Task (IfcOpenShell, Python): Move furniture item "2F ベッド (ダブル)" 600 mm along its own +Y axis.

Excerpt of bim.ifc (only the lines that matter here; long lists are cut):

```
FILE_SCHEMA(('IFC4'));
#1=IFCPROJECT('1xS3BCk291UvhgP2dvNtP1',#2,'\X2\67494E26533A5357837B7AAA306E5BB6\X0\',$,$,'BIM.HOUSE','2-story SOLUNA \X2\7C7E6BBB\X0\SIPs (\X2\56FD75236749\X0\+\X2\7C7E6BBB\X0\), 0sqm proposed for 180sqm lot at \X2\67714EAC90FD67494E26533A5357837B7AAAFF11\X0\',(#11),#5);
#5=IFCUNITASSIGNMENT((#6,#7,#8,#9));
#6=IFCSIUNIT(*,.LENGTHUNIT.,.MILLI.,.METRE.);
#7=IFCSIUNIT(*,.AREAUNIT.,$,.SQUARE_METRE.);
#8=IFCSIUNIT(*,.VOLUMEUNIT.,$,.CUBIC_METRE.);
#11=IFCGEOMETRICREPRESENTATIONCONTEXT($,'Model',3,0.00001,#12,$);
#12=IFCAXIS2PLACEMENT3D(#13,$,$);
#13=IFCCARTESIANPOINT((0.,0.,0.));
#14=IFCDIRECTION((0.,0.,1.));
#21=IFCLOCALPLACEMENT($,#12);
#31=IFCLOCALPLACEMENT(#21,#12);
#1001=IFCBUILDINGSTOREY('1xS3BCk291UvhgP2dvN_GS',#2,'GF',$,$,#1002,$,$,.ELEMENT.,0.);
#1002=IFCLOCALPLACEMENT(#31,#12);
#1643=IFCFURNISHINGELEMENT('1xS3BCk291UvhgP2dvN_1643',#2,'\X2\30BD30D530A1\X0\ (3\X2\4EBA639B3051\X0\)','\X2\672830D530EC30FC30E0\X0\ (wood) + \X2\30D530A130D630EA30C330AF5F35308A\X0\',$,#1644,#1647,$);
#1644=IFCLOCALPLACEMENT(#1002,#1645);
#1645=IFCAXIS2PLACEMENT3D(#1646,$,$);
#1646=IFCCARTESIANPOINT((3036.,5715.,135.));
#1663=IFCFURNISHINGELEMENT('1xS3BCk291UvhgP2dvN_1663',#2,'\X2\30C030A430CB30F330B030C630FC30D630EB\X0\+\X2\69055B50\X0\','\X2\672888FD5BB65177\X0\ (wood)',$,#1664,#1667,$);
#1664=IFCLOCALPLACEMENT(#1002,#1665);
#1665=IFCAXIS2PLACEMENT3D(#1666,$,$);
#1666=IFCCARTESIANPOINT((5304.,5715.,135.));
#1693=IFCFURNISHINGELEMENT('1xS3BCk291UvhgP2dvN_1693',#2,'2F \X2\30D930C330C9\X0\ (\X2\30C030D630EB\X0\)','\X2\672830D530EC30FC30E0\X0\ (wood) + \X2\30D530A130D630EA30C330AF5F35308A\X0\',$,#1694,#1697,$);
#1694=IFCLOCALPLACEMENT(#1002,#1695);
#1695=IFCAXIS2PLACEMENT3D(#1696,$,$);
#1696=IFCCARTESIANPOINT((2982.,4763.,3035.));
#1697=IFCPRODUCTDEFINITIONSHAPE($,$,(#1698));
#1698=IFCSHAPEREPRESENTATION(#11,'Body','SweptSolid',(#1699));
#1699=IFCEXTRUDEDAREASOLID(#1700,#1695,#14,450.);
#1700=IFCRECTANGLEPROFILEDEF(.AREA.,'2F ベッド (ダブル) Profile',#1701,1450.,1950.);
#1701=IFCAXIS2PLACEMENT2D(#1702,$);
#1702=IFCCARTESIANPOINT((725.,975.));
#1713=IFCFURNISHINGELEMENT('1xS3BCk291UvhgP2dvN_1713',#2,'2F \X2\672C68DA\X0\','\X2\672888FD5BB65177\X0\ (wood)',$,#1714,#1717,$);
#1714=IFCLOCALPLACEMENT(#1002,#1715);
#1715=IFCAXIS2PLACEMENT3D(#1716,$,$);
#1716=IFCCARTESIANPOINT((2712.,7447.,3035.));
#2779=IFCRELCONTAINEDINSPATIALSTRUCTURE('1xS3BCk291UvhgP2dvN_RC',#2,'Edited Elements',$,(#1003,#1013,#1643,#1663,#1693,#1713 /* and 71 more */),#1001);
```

```python
import ifcopenshell
import ifcopenshell.api.geometry
import ifcopenshell.util.placement

model = ifcopenshell.open("bim.ifc")

item = model.by_guid("1xS3BCk291UvhgP2dvN_1693")
matrix = ifcopenshell.util.placement.get_local_placement(item.ObjectPlacement)
matrix[:3, 3] += matrix[:3, 1] * 600.0
ifcopenshell.api.geometry.edit_object_placement(model, product=item, matrix=matrix, is_si=False)

print(ifcopenshell.util.placement.get_local_placement(item.ObjectPlacement).round(3) + 0.0)

model.write("bim_v2.ifc")
```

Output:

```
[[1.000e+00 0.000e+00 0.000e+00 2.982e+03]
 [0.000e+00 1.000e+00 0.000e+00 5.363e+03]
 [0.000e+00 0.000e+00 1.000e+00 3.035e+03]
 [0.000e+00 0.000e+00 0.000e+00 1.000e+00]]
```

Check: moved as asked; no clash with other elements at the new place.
